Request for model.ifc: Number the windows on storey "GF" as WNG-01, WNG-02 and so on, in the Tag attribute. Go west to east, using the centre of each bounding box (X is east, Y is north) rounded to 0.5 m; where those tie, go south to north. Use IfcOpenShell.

First a look at what the model holds.

```python
import ifcopenshell
import ifcopenshell.util.element
import ifcopenshell.util.placement

model = ifcopenshell.open("model.ifc")
print(model.schema)
storey = next(s for s in model.by_type("IfcBuildingStorey") if s.Name == "GF")
windows = [e for e in ifcopenshell.util.element.get_decomposition(storey) if e.is_a("IfcWindow")]
for e in sorted(windows, key=lambda e: e.id()):
    origin = ifcopenshell.util.placement.get_local_placement(e.ObjectPlacement)[:3, 3]
    print(e.id(), e.Tag, e.Name, origin.round(2) + 0.0, sep=" | ")
```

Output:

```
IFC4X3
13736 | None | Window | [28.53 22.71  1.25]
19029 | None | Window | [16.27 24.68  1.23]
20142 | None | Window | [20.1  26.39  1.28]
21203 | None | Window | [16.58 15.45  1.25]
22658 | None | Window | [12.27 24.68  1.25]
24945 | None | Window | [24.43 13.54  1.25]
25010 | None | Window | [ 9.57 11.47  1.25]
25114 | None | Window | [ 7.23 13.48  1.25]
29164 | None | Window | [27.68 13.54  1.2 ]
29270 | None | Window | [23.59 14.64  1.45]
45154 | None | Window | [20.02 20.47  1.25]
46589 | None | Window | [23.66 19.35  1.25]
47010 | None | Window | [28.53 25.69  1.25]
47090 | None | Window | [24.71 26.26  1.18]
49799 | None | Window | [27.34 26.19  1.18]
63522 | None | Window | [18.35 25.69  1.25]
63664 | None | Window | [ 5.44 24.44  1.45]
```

```python
import ifcopenshell
import ifcopenshell.geom
import ifcopenshell.util.element
import ifcopenshell.util.shape

model = ifcopenshell.open("model.ifc")
settings = ifcopenshell.geom.settings()
settings.set("use-world-coords", True)


def centre(element):
    shape = ifcopenshell.geom.create_shape(settings, element)
    return ifcopenshell.util.shape.get_bbox_centroid(shape.geometry)


storey = next(s for s in model.by_type("IfcBuildingStorey") if s.Name == "GF")
windows = [e for e in ifcopenshell.util.element.get_decomposition(storey) if e.is_a("IfcWindow")]

# Insertion points can sit at a corner or the storey origin, so sort by the geometry (in metres).
centres = {e: centre(e) for e in windows}
windows.sort(key=lambda e: (round(centres[e][0] / 0.5), centres[e][1]))

for i, e in enumerate(windows, start=1):
    number = f"WNG-{i:02d}"
    e.Tag = number
    print(e.id(), number)

model.write("model-out.ifc")
```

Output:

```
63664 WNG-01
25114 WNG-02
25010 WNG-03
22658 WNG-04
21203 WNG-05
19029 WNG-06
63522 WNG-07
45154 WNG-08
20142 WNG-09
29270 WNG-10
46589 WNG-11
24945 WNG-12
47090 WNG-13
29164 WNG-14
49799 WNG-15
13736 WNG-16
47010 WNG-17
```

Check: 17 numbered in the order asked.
